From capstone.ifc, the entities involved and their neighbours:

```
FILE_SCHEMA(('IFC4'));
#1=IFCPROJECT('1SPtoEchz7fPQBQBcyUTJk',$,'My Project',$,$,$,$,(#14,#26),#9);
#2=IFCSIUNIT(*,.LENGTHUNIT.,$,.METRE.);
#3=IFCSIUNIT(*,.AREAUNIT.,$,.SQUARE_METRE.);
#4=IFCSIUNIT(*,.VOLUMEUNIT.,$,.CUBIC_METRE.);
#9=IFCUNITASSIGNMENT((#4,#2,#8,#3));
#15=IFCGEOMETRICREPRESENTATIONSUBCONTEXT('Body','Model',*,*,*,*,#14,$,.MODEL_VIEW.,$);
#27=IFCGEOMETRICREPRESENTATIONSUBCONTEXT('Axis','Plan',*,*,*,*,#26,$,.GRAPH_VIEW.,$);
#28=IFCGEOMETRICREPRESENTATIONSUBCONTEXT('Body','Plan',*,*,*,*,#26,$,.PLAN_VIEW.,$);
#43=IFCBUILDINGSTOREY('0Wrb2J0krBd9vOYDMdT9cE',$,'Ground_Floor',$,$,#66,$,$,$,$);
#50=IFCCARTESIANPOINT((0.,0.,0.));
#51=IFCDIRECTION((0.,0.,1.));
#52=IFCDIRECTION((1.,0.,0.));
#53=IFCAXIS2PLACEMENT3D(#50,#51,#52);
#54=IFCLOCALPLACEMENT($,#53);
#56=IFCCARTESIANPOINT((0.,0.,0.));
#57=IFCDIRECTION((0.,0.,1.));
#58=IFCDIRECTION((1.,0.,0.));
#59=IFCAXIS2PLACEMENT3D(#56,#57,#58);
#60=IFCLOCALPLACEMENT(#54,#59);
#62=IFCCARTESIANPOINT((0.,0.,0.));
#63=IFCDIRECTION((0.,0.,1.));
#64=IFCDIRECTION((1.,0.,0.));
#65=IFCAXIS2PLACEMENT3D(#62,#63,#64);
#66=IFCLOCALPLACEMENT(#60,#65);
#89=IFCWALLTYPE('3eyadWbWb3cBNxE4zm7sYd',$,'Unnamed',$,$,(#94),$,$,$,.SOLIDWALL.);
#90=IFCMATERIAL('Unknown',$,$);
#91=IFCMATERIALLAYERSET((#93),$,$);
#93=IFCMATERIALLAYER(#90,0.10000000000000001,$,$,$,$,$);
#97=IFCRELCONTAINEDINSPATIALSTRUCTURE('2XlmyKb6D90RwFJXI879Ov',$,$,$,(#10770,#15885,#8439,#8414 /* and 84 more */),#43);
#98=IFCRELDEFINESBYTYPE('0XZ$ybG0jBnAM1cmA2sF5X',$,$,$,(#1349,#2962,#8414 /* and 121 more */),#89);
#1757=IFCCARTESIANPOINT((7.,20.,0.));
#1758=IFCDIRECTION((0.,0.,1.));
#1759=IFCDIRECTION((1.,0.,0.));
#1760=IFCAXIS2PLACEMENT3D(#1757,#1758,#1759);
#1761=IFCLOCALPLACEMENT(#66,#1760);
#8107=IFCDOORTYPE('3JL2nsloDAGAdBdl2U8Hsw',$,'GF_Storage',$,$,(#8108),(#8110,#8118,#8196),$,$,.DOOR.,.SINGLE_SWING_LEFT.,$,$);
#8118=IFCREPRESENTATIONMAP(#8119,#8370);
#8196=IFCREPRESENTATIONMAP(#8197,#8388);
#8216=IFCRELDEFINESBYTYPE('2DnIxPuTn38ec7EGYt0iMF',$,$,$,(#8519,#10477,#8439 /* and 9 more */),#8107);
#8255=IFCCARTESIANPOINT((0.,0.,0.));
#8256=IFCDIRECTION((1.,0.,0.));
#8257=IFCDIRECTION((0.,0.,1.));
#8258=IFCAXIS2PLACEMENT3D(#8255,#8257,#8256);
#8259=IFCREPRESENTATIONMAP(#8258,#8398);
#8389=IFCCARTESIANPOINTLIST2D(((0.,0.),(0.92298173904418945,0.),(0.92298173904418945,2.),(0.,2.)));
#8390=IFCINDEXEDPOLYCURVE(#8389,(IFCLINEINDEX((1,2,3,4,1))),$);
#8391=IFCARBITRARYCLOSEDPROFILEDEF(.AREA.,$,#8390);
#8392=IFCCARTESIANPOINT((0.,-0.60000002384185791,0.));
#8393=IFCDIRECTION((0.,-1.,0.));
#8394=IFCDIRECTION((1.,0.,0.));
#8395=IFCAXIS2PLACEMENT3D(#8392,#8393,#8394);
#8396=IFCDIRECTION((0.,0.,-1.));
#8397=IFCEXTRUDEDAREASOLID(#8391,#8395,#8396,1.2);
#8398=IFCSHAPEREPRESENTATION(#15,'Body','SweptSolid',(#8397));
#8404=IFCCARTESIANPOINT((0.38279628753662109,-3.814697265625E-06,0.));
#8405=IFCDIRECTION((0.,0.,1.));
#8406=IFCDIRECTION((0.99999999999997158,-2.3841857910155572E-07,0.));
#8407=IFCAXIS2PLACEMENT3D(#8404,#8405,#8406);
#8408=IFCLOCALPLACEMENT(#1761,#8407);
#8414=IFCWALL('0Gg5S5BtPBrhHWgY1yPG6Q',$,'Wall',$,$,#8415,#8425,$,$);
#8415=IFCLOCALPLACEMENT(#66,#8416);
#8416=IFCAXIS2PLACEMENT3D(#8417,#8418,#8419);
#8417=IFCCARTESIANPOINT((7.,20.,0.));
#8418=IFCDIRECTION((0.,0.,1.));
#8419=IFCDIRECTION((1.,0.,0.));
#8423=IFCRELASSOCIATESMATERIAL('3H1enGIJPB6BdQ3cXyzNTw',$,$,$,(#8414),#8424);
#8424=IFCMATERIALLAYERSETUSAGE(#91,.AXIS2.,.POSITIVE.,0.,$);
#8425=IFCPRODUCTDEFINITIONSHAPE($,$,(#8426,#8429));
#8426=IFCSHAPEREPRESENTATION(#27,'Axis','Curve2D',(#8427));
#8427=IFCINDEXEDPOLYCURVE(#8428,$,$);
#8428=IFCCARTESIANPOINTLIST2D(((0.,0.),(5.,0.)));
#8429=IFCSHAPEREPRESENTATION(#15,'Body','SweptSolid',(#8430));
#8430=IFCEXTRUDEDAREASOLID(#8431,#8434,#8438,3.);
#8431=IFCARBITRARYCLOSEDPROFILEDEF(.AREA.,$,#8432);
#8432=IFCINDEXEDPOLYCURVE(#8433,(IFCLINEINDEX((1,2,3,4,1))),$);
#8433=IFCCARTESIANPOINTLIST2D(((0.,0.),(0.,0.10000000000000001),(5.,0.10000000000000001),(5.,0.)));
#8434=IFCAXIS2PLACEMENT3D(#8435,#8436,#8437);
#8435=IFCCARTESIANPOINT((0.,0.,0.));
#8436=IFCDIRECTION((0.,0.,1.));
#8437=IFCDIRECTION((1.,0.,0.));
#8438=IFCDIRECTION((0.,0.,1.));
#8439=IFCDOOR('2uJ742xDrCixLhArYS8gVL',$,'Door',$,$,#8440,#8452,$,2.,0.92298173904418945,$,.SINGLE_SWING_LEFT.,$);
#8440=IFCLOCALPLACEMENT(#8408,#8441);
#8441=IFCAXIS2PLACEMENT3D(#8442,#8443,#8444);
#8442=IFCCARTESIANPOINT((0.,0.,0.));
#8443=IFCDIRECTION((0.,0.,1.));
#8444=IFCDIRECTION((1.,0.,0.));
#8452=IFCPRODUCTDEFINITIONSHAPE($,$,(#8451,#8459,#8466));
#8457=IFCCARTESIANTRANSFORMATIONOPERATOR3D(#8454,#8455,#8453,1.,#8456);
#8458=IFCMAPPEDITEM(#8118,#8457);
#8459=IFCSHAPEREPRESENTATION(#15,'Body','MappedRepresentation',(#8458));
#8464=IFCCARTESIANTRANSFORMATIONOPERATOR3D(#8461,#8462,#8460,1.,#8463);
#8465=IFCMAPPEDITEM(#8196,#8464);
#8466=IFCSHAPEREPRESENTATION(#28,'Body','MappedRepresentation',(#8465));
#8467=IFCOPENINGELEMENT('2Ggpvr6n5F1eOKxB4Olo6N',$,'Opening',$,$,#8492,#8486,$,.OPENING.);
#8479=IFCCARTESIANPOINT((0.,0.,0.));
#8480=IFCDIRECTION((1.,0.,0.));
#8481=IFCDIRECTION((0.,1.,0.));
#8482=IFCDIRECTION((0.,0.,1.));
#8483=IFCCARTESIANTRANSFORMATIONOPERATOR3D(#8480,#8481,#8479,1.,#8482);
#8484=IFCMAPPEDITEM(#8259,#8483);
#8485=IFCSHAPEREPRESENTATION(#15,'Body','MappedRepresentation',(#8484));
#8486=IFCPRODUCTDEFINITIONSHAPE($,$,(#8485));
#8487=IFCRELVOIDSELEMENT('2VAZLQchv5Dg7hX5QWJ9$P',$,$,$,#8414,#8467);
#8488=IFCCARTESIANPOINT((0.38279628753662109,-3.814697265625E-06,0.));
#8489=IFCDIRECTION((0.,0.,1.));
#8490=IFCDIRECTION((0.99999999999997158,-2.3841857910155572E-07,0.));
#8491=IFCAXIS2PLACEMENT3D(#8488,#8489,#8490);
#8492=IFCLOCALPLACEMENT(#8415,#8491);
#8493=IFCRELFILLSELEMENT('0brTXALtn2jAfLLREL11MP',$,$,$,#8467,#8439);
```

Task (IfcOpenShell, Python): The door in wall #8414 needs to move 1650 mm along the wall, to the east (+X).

```python
import ifcopenshell
import ifcopenshell.api.geometry
import ifcopenshell.util.placement
import ifcopenshell.util.unit

model = ifcopenshell.open("capstone.ifc")
unit_scale = ifcopenshell.util.unit.calculate_unit_scale(model)

door = model.by_guid("2uJ742xDrCixLhArYS8gVL")
opening = door.FillsVoids[0].RelatingOpeningElement
wall = opening.VoidsElements[0].RelatingBuildingElement

wall_matrix = ifcopenshell.util.placement.get_local_placement(wall.ObjectPlacement)
shift = wall_matrix[:3, 0] * 1.65 / unit_scale
before = ifcopenshell.util.placement.get_local_placement(door.ObjectPlacement)[:3, 3].copy()

# The door is not placed relative to its opening, so move both.
for product in (opening, door):
    matrix = ifcopenshell.util.placement.get_local_placement(product.ObjectPlacement)
    matrix[:3, 3] += shift
    ifcopenshell.api.geometry.edit_object_placement(model, product=product, matrix=matrix, is_si=False)

after = ifcopenshell.util.placement.get_local_placement(door.ObjectPlacement)[:3, 3]
print("door moved by", (after - before).round(3) + 0.0)

model.write("capstone-out.ifc")
```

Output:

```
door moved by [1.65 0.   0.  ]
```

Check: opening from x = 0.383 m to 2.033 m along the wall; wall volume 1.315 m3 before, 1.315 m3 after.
